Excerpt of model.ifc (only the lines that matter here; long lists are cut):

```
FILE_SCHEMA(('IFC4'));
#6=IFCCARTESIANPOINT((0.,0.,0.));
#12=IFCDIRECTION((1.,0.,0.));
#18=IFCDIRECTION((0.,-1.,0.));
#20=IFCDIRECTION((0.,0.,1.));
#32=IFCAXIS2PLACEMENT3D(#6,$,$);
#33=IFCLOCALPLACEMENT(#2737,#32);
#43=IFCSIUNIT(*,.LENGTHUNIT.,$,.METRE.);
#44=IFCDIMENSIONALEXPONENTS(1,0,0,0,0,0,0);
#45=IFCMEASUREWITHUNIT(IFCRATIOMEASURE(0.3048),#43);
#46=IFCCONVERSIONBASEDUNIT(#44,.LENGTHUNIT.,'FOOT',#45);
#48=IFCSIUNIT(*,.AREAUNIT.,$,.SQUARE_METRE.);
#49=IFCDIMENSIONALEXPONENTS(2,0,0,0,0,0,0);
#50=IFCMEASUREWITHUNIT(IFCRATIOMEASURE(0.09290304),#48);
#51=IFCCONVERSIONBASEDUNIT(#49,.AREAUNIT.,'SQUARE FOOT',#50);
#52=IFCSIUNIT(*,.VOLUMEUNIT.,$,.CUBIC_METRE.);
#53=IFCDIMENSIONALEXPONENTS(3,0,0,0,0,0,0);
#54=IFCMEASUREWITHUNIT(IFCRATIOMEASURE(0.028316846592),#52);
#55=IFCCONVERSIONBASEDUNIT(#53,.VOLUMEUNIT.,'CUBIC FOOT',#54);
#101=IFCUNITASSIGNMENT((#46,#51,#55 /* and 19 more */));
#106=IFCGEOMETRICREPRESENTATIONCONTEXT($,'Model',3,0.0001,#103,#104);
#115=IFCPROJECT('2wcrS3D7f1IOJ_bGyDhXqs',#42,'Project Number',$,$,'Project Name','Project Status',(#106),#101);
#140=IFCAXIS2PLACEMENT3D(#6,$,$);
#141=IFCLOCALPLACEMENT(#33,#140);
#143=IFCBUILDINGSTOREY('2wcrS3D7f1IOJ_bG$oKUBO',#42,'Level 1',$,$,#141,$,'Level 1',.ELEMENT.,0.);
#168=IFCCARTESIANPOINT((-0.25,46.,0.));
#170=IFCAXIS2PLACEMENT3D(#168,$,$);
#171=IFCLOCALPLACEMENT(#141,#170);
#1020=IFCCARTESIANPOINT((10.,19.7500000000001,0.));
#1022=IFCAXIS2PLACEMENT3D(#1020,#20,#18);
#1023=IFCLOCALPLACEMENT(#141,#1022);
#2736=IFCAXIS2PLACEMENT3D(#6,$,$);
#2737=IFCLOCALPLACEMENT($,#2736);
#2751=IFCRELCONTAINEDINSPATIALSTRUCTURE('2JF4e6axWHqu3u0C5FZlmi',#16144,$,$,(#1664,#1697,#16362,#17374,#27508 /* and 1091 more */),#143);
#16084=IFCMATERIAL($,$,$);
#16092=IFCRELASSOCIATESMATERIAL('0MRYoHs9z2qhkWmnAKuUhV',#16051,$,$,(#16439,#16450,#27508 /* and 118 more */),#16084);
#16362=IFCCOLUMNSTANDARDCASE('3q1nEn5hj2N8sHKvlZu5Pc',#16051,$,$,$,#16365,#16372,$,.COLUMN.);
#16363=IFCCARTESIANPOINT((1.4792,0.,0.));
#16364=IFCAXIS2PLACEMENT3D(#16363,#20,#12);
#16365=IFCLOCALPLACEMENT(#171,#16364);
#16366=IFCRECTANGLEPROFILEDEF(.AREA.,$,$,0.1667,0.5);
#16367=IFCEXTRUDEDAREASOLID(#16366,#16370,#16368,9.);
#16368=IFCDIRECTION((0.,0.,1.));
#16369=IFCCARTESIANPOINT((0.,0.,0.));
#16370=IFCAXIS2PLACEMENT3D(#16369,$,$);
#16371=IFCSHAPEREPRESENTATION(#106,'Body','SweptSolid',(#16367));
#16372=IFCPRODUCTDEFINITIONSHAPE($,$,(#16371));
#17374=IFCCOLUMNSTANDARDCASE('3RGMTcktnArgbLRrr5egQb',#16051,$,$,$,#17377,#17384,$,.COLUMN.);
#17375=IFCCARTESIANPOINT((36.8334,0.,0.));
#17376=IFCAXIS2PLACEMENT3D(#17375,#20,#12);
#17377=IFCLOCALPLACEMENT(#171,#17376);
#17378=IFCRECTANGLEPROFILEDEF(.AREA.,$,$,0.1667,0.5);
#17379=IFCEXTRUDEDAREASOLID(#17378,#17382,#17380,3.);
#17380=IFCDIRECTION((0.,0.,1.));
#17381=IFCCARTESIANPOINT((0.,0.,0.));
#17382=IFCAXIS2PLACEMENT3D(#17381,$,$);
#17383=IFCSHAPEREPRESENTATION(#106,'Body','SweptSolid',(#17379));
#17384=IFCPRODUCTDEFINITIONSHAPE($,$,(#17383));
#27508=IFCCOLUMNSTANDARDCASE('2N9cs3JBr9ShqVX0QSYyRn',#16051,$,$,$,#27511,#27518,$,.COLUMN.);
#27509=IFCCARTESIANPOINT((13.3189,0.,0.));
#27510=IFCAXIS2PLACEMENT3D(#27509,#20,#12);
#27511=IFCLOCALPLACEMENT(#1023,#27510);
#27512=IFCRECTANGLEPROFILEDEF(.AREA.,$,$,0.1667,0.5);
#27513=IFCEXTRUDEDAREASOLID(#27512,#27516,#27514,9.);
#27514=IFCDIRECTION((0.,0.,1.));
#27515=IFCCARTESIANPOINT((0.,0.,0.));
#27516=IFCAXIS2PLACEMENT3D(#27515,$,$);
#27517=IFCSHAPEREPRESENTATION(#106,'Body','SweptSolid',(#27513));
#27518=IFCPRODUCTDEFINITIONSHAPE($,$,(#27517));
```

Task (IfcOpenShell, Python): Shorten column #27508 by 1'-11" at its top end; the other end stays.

```python
import ifcopenshell
import ifcopenshell.util.unit

model = ifcopenshell.open("model.ifc")
unit_scale = ifcopenshell.util.unit.calculate_unit_scale(model)

member = model.by_id(27508)
change = -23 * 0.0254 / unit_scale

# The extrusion runs towards the end named, so only its depth changes.
body = next(r for r in member.Representation.Representations if r.RepresentationIdentifier == "Body")
solid = body.Items[0]
old_length = solid.Depth
solid.Depth += change

print(f"length {old_length:g} -> {solid.Depth:g}")

model.write("model_v2.ifc")
```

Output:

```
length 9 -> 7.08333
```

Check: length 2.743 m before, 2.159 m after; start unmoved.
